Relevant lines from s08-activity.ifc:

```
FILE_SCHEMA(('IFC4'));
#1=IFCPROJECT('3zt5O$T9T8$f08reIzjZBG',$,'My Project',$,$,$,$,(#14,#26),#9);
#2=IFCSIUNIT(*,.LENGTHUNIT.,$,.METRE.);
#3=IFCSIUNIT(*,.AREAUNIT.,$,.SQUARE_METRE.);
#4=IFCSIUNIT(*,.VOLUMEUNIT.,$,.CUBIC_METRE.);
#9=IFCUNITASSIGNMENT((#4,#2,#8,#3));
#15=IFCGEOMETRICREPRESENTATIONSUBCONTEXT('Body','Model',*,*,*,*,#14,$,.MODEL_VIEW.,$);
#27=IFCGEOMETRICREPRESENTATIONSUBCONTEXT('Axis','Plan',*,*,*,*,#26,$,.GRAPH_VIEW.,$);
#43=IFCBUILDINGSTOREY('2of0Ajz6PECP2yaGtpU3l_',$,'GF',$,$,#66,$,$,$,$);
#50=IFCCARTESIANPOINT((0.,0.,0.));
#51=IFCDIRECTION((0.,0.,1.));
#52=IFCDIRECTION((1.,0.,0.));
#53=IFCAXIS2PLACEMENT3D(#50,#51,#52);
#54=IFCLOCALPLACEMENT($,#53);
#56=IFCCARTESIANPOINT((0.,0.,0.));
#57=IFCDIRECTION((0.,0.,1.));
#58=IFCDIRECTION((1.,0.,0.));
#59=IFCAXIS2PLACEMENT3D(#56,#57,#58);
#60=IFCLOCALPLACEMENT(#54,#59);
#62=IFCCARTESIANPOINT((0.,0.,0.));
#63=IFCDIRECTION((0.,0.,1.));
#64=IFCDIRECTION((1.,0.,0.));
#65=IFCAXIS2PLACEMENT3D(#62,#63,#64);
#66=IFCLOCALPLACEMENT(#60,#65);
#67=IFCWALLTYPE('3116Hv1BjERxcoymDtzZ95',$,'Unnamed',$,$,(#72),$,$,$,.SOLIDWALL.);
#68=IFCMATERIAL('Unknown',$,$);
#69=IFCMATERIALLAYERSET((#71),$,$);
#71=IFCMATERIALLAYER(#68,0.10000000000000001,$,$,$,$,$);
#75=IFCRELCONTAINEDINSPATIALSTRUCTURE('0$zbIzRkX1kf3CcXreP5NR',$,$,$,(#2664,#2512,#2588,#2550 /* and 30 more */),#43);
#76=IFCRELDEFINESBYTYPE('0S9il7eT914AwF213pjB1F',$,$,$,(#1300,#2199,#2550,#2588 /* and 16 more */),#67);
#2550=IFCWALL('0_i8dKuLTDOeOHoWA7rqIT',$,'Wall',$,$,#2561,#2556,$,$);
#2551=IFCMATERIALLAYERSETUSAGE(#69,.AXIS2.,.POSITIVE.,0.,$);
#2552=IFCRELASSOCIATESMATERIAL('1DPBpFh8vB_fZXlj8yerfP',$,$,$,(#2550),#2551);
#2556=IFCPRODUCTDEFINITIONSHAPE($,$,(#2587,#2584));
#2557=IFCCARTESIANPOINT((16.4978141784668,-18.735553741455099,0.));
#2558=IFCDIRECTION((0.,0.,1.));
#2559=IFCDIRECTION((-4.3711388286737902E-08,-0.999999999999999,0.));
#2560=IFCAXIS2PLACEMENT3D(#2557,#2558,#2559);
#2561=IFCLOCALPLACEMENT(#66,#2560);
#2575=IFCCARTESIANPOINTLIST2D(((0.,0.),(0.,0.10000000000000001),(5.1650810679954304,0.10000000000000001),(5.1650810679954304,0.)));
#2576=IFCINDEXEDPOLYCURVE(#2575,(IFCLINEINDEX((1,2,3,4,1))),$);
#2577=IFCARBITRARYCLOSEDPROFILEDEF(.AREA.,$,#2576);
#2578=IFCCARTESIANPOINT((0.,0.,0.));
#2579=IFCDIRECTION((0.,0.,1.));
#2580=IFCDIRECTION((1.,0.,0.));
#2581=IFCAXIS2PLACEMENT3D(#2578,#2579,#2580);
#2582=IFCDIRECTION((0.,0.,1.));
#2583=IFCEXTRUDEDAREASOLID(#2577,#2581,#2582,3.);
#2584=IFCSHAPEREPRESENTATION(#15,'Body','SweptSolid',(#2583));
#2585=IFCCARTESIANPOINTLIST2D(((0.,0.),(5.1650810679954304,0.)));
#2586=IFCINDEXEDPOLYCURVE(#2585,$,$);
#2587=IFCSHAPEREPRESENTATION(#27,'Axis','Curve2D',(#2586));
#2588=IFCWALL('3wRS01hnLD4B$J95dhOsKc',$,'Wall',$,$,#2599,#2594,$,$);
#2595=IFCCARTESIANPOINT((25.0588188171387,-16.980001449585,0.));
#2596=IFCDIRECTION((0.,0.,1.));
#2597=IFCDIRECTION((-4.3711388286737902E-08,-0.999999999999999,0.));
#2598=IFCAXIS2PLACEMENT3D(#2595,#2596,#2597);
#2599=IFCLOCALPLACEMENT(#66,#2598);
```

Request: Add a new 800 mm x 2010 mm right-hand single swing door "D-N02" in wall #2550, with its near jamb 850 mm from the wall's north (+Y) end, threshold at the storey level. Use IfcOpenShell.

```python
import numpy as np
import ifcopenshell
import ifcopenshell.api.feature
import ifcopenshell.api.geometry
import ifcopenshell.api.root
import ifcopenshell.api.spatial
import ifcopenshell.geom
import ifcopenshell.util.element
import ifcopenshell.util.placement
import ifcopenshell.util.representation
import ifcopenshell.util.shape
import ifcopenshell.util.unit

model = ifcopenshell.open("s08-activity.ifc")
unit_scale = ifcopenshell.util.unit.calculate_unit_scale(model)
settings = ifcopenshell.geom.settings()


def volume(element):
    """Net volume in cubic metres, openings subtracted."""
    shape = ifcopenshell.geom.create_shape(settings, element)
    return ifcopenshell.util.shape.get_volume(shape.geometry)


wall = model.by_id(2550)
storey = ifcopenshell.util.element.get_container(wall, ifc_class="IfcBuildingStorey")
context = ifcopenshell.util.representation.get_context(model, "Model", "Body", "MODEL_VIEW")
before = volume(wall)

width, height, from_end, sill = 0.8, 2.01, 0.85, 0.0  # metres

# The wall runs along its own X axis, and the end named is its -X end.
wall_shape = ifcopenshell.geom.create_shape(settings, wall)
x, y, z = ifcopenshell.util.shape.get_vertices(wall_shape.geometry).T
start = x.min() + from_end
face, thickness = float(y.min()), float(y.max() - y.min())
wall_matrix = ifcopenshell.util.placement.get_local_placement(wall.ObjectPlacement)
level = ifcopenshell.util.placement.get_local_placement(storey.ObjectPlacement)[2, 3]


def in_wall(x, y):
    """Placement at x, y metres in the wall's axes, at sill height."""
    matrix = wall_matrix.copy()
    matrix[:, 3] = wall_matrix @ np.array([x / unit_scale, y / unit_scale, 0.0, 1.0])
    matrix[2, 3] = level + sill / unit_scale
    return matrix


# Opening: a box that overshoots both wall faces by 50 mm.
opening = ifcopenshell.api.root.create_entity(model, ifc_class="IfcOpeningElement", predefined_type="OPENING")
box = ifcopenshell.api.geometry.add_wall_representation(
    model, context=context, length=width, height=height, thickness=thickness + 0.1
)
ifcopenshell.api.geometry.assign_representation(model, product=opening, representation=box)
ifcopenshell.api.geometry.edit_object_placement(model, product=opening, matrix=in_wall(start, face - 0.05), is_si=False)
ifcopenshell.api.feature.add_feature(model, feature=opening, element=wall)

door = ifcopenshell.api.root.create_entity(model, ifc_class="IfcDoor", name="D-N02", predefined_type="DOOR")
door.OverallWidth, door.OverallHeight = width / unit_scale, height / unit_scale
door.OperationType = "SINGLE_SWING_RIGHT"
body = ifcopenshell.api.geometry.add_door_representation(
    model,
    context=context,
    overall_width=door.OverallWidth,
    overall_height=door.OverallHeight,
    operation_type="SINGLE_SWING_RIGHT",
    lining_properties={"LiningDepth": thickness / unit_scale, "ThresholdDepth": thickness / unit_scale},
)
ifcopenshell.api.geometry.assign_representation(model, product=door, representation=body)
ifcopenshell.api.spatial.assign_container(model, products=[door], relating_structure=storey)
ifcopenshell.api.feature.add_filling(model, opening=opening, element=door)

# The lining spans the wall, so the door starts at the wall face.
ifcopenshell.api.geometry.edit_object_placement(model, product=door, matrix=in_wall(start, face), is_si=False)

after = volume(wall)

print(f"wall volume {before:.3f} -> {after:.3f} m3")

model.write("s08-activity_edited.ifc")
```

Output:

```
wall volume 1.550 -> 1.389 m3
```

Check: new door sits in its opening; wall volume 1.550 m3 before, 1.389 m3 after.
